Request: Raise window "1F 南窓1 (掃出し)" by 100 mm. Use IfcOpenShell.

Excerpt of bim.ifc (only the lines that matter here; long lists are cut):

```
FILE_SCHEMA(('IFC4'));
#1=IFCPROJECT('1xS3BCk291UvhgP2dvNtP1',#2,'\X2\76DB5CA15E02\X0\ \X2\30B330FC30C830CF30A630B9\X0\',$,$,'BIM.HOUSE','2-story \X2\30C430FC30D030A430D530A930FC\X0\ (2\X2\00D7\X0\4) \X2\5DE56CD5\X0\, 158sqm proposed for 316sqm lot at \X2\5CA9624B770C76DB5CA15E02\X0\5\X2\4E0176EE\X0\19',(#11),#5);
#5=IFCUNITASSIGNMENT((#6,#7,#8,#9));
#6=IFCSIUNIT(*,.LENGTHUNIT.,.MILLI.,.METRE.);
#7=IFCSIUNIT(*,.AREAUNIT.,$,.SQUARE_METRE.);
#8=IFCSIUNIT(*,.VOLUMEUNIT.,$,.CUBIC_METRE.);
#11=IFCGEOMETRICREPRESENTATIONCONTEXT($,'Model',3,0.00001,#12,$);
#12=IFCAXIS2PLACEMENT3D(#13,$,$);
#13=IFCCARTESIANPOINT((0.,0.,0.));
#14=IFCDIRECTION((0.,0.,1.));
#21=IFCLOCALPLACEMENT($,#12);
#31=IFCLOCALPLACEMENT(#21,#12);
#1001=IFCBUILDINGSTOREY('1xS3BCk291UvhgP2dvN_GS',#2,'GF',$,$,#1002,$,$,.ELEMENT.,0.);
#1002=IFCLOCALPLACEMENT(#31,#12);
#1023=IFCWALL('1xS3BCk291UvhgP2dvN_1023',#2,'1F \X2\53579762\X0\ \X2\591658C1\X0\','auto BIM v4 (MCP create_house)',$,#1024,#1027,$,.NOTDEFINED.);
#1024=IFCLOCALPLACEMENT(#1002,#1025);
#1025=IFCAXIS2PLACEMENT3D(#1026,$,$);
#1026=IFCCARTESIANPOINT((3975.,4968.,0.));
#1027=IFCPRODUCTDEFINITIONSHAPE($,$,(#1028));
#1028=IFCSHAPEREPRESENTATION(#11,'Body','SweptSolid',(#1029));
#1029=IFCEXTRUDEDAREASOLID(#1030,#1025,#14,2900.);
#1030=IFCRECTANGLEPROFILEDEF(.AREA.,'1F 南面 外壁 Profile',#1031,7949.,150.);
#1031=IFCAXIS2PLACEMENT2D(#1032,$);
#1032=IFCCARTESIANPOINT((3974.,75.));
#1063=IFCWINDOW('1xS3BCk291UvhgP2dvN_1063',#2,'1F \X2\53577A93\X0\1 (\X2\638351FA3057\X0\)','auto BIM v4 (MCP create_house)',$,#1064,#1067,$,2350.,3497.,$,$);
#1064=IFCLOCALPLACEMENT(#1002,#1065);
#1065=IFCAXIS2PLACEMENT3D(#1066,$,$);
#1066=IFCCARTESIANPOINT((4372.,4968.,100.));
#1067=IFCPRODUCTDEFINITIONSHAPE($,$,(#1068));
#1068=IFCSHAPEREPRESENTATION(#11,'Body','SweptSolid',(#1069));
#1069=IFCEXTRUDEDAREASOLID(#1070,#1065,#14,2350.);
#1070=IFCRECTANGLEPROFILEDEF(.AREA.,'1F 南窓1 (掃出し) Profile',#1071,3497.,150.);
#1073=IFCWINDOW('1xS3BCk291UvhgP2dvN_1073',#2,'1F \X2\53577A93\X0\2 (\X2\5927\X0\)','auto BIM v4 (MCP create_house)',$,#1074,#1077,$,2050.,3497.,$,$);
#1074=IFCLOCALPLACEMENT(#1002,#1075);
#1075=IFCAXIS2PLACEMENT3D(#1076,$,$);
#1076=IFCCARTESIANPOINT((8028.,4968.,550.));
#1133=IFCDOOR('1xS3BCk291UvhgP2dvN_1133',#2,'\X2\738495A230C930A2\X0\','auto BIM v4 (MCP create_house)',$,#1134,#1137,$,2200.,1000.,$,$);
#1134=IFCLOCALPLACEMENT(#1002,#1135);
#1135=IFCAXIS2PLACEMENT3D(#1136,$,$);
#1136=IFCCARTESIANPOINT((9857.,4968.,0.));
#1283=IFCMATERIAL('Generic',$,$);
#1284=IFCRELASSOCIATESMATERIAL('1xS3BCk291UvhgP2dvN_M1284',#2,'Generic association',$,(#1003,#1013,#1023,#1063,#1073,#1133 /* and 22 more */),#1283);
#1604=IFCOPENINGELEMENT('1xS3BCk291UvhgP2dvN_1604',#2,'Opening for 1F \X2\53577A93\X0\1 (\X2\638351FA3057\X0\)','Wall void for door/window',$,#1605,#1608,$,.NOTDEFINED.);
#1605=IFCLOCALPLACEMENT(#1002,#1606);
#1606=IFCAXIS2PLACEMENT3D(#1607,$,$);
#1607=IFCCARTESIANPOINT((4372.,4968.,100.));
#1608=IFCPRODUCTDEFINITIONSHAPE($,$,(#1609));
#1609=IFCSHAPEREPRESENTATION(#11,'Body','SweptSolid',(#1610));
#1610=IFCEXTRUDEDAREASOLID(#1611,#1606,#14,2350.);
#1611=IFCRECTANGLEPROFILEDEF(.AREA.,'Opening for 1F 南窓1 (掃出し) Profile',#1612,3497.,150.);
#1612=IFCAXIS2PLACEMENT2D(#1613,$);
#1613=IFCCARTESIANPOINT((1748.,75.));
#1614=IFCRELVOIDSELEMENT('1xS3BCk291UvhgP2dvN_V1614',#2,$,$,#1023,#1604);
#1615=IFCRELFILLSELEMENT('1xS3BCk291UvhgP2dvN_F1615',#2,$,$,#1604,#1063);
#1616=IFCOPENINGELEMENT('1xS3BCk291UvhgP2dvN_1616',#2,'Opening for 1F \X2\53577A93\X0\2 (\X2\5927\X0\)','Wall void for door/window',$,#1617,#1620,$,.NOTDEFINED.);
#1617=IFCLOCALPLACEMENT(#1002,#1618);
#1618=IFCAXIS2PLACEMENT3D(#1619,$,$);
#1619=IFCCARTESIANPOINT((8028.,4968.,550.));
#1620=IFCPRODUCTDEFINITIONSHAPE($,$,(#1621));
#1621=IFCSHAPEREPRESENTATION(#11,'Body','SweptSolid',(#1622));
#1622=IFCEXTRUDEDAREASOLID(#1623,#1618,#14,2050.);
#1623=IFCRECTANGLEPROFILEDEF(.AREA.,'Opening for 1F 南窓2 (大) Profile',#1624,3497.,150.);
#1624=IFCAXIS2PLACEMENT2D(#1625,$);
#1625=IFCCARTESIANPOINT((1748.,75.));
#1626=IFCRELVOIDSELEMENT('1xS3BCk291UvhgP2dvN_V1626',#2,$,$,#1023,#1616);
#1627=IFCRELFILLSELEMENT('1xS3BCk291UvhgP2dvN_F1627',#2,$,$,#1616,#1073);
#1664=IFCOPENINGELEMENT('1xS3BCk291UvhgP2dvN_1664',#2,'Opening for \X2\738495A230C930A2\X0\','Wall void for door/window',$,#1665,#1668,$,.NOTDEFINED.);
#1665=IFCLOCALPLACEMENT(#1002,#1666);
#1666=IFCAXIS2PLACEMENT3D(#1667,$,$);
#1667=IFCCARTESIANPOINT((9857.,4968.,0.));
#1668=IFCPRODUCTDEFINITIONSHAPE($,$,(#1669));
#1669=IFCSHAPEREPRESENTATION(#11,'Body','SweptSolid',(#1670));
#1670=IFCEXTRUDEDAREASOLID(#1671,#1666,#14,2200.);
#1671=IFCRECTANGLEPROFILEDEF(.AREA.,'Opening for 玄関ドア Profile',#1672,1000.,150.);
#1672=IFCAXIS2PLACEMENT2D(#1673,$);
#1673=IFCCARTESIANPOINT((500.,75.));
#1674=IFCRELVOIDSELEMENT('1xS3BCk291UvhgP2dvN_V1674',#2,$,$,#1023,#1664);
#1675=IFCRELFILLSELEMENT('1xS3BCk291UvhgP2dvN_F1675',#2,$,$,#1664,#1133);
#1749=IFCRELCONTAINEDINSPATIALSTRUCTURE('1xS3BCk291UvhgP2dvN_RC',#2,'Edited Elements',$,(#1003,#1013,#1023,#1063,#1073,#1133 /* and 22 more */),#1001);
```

```python
import numpy as np
import ifcopenshell
import ifcopenshell.api.geometry
import ifcopenshell.util.placement
import ifcopenshell.util.unit

model = ifcopenshell.open("bim.ifc")
unit_scale = ifcopenshell.util.unit.calculate_unit_scale(model)

window = model.by_guid("1xS3BCk291UvhgP2dvN_1063")
opening = window.FillsVoids[0].RelatingOpeningElement
dz = 0.1 / unit_scale

shift = np.array([0.0, 0.0, dz])
# The window is not placed relative to its opening, so move both.
for product in (opening, window):
    matrix = ifcopenshell.util.placement.get_local_placement(product.ObjectPlacement)
    matrix[:3, 3] += shift
    ifcopenshell.api.geometry.edit_object_placement(model, product=product, matrix=matrix, is_si=False)

print(f"moved by {dz * unit_scale:+.3f} m")

model.write("bim-out.ifc")
```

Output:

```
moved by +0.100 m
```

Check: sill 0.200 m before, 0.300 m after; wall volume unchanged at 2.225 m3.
